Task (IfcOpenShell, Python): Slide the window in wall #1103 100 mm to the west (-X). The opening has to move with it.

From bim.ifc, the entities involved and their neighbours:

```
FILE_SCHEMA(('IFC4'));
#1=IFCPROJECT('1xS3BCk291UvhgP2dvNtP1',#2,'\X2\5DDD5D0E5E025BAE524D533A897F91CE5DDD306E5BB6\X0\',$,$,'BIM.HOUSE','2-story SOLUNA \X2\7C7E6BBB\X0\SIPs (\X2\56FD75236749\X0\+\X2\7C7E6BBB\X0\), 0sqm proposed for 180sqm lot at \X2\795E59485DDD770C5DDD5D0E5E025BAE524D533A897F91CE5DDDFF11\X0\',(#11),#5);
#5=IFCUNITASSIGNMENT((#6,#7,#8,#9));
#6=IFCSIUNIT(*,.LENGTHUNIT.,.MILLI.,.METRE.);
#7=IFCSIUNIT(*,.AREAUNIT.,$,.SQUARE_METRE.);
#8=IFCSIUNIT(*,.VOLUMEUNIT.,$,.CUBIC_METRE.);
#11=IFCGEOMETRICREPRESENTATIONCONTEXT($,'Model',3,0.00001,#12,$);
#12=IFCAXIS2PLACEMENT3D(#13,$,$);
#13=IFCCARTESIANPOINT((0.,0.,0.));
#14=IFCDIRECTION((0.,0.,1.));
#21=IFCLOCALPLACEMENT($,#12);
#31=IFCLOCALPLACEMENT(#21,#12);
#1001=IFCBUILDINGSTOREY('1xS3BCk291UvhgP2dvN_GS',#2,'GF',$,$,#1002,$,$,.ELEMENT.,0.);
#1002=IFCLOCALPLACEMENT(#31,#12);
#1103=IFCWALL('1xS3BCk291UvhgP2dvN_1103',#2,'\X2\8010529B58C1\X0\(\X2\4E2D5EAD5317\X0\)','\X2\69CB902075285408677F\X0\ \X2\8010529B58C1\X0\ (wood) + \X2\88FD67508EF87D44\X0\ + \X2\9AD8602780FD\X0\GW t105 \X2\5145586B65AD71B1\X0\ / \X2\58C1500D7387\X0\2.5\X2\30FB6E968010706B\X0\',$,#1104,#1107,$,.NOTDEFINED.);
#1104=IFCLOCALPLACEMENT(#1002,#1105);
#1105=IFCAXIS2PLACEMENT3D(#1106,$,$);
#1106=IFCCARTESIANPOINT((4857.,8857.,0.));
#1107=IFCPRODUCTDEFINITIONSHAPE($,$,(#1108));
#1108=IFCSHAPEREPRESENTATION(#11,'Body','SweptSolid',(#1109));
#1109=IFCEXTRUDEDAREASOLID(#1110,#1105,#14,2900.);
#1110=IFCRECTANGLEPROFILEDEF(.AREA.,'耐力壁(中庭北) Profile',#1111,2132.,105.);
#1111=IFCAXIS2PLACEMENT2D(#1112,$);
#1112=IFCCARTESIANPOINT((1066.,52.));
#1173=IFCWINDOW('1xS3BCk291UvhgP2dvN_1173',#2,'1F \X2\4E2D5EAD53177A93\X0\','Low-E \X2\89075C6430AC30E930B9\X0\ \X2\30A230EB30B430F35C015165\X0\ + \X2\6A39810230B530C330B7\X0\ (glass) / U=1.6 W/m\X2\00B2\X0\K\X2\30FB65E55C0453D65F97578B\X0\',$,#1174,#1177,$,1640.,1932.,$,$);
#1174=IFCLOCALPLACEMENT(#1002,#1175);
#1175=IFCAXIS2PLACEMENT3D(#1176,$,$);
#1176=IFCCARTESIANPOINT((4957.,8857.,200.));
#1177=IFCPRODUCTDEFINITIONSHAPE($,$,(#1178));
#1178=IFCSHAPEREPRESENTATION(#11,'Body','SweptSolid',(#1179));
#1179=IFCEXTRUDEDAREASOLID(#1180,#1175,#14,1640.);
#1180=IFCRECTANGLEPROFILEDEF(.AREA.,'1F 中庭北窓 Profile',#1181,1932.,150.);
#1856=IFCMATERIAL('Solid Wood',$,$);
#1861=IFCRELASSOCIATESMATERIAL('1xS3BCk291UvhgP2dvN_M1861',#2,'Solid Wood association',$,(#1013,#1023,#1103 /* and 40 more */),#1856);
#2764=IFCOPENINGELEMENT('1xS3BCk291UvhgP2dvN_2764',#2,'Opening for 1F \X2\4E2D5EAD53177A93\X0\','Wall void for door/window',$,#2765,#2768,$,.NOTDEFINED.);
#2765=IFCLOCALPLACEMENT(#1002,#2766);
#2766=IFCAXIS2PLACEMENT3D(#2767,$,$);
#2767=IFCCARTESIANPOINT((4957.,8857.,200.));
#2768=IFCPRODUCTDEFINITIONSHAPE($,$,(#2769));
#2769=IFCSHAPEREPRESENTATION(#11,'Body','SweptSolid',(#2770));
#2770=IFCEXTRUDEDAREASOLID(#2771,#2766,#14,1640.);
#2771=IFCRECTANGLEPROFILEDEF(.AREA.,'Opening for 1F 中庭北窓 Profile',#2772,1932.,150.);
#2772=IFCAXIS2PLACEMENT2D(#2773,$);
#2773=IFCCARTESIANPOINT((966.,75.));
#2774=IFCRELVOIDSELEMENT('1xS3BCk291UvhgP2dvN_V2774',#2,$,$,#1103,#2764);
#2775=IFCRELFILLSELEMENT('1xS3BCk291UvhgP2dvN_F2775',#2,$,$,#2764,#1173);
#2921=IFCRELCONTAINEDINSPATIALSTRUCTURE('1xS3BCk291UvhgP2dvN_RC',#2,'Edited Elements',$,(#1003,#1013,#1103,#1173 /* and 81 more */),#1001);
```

```python
import ifcopenshell
import ifcopenshell.api.geometry
import ifcopenshell.util.placement
import ifcopenshell.util.unit

model = ifcopenshell.open("bim.ifc")
unit_scale = ifcopenshell.util.unit.calculate_unit_scale(model)

window = model.by_guid("1xS3BCk291UvhgP2dvN_1173")
opening = window.FillsVoids[0].RelatingOpeningElement
wall = opening.VoidsElements[0].RelatingBuildingElement

wall_matrix = ifcopenshell.util.placement.get_local_placement(wall.ObjectPlacement)
shift = wall_matrix[:3, 0] * -0.1 / unit_scale
before = ifcopenshell.util.placement.get_local_placement(window.ObjectPlacement)[:3, 3].copy()

# The window is not placed relative to its opening, so move both.
for product in (opening, window):
    matrix = ifcopenshell.util.placement.get_local_placement(product.ObjectPlacement)
    matrix[:3, 3] += shift
    ifcopenshell.api.geometry.edit_object_placement(model, product=product, matrix=matrix, is_si=False)

after = ifcopenshell.util.placement.get_local_placement(window.ObjectPlacement)[:3, 3]
print("window moved by", (after - before).round(3) + 0.0)

model.write("bim_updated.ifc")
```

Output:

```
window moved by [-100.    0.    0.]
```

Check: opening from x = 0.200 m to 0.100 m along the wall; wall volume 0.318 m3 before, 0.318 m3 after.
